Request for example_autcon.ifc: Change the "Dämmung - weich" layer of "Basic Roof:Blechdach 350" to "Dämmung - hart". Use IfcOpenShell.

First a look at what the model holds.

```python
import ifcopenshell
import ifcopenshell.util.element

model = ifcopenshell.open("example_autcon.ifc")
print(model.schema)
for layer_set in model.by_type("IfcMaterialLayerSet"):
    if layer_set.LayerSetName == "Basic Roof:Blechdach 350":
        for layer in layer_set.MaterialLayers:
            print(layer.id(), layer.Material and layer.Material.Name, layer.LayerThickness, sep=" | ")
        print(len(ifcopenshell.util.element.get_elements_by_material(model, layer_set)), "elements and types use it")
print(sorted(m.Name for m in model.by_type("IfcMaterial") if m.Name)[:60])
```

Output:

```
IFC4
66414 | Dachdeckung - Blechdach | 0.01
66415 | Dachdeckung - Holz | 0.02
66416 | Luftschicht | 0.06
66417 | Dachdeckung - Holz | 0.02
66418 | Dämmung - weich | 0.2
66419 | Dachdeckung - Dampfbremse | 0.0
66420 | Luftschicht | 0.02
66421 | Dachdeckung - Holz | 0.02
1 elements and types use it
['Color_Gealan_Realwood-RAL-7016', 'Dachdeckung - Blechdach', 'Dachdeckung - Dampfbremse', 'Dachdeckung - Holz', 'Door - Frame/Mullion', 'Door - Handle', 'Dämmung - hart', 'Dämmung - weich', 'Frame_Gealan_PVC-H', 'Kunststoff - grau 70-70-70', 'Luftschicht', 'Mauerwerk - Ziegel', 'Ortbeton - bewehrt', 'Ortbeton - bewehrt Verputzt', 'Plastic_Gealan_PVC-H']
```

```python
import ifcopenshell
import ifcopenshell.api.material

model = ifcopenshell.open("example_autcon.ifc")

layer_set = next(s for s in model.by_type("IfcMaterialLayerSet") if s.LayerSetName == "Basic Roof:Blechdach 350")
layer = next(l for l in layer_set.MaterialLayers if l.Material and l.Material.Name == "Dämmung - weich")
material = next(m for m in model.by_type("IfcMaterial") if m.Name == "Dämmung - hart")

# Point this one layer at the other material; renaming the old one would change it everywhere.
ifcopenshell.api.material.edit_layer(model, layer=layer, attributes={"Name": material.Name}, material=material)

print([l.Material.Name if l.Material else None for l in layer_set.MaterialLayers])

model.write("example_autcon_v2.ifc")
```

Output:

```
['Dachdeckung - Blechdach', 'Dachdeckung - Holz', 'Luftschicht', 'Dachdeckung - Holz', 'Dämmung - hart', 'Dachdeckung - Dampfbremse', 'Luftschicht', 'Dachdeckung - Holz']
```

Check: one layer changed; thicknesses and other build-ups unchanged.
